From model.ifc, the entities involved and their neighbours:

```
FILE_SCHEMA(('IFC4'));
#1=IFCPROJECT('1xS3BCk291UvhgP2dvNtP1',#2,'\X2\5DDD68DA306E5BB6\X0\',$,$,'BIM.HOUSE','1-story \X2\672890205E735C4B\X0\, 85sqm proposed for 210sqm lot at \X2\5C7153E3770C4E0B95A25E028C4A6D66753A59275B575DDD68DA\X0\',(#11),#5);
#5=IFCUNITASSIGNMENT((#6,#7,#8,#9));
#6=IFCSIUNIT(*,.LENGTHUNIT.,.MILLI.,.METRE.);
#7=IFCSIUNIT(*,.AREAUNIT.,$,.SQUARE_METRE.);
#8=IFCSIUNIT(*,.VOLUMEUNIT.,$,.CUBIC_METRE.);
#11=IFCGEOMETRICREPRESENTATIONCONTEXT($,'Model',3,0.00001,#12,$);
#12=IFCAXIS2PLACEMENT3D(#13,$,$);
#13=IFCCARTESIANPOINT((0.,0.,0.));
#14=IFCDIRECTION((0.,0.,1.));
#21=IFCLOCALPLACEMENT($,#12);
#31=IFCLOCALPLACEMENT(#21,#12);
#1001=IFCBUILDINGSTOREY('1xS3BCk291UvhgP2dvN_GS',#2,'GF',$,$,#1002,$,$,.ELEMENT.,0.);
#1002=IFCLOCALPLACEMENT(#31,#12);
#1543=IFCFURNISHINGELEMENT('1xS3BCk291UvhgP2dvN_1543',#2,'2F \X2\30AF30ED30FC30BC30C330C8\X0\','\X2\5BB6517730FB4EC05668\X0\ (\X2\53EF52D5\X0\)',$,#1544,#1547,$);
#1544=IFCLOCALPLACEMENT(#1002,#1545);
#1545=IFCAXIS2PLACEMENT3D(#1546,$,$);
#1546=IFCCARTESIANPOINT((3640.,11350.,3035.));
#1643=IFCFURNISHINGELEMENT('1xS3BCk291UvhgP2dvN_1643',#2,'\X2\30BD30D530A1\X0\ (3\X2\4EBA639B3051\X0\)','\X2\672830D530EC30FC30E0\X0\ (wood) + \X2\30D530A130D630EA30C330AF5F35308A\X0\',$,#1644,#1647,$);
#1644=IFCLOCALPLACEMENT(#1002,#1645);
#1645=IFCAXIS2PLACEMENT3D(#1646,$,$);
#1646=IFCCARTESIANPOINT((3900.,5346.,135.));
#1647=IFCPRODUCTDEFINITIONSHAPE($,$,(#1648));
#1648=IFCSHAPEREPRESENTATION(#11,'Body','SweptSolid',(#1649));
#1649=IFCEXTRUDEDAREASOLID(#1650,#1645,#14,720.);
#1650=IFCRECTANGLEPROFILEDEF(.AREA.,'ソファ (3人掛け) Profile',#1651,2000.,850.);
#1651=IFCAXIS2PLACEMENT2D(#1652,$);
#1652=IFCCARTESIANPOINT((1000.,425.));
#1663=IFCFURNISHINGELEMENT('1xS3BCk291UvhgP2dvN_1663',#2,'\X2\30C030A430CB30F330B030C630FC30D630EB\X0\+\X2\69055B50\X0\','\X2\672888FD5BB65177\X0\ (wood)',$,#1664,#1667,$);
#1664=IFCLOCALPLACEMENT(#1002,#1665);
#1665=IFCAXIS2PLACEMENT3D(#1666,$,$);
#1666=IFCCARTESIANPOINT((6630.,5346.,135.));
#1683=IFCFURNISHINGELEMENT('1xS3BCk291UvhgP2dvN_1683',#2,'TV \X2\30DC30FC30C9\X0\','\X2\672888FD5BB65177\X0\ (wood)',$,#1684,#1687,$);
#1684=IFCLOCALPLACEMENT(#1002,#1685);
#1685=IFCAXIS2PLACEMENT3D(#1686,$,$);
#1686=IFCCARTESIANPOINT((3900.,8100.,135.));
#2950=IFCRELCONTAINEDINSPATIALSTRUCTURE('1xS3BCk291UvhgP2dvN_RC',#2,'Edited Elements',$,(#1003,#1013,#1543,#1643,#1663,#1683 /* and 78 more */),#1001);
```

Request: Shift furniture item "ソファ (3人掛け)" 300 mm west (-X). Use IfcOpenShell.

```python
import ifcopenshell
import ifcopenshell.api.geometry
import ifcopenshell.util.placement
import ifcopenshell.util.unit

model = ifcopenshell.open("model.ifc")
unit_scale = ifcopenshell.util.unit.calculate_unit_scale(model)

item = model.by_guid("1xS3BCk291UvhgP2dvN_1643")
matrix = ifcopenshell.util.placement.get_local_placement(item.ObjectPlacement)
matrix[0, 3] -= 0.3 / unit_scale
ifcopenshell.api.geometry.edit_object_placement(model, product=item, matrix=matrix, is_si=False)

print(ifcopenshell.util.placement.get_local_placement(item.ObjectPlacement).round(3) + 0.0)

model.write("model_updated.ifc")
```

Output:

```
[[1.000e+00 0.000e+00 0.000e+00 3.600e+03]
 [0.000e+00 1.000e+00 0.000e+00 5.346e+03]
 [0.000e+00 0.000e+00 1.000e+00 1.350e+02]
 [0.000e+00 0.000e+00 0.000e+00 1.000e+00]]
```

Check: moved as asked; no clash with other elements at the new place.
